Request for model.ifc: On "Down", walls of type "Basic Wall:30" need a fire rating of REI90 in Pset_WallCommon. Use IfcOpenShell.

First a look at what the model holds.

```python
import ifcopenshell
import ifcopenshell.util.element

model = ifcopenshell.open("model.ifc")
print(model.schema)
storey = next(s for s in model.by_type("IfcBuildingStorey") if s.Name == "Down")
walls = [e for e in ifcopenshell.util.element.get_decomposition(storey) if e.is_a("IfcWall")]
seen = {}
for e in walls:
    element_type = ifcopenshell.util.element.get_type(e)
    key = (element_type.Name if element_type != e and element_type else None, ifcopenshell.util.element.get_pset(e, "Pset_WallCommon", "FireRating"))
    seen[key] = seen.get(key, 0) + 1
for (name, value), count in sorted(seen.items(), key=str):
    print(count, "x", name, "|", value)
```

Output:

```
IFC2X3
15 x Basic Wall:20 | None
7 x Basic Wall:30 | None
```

```python
import ifcopenshell
import ifcopenshell.api.pset
import ifcopenshell.util.element

model = ifcopenshell.open("model.ifc")

storey = next(s for s in model.by_type("IfcBuildingStorey") if s.Name == "Down")
walls = [e for e in ifcopenshell.util.element.get_decomposition(storey) if e.is_a("IfcWall")]

count = 0
for e in walls:
    element_type = ifcopenshell.util.element.get_type(e)
    if element_type in (None, e) or element_type.Name != "Basic Wall:30":
        continue
    # add_pset returns the element's existing set when there is one.
    pset = ifcopenshell.api.pset.add_pset(model, product=e, name="Pset_WallCommon")
    ifcopenshell.api.pset.edit_pset(model, pset=pset, properties={"FireRating": "REI90"})
    count += 1

print(count, "walls updated")

model.write("model_v2.ifc")
```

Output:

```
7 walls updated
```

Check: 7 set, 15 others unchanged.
